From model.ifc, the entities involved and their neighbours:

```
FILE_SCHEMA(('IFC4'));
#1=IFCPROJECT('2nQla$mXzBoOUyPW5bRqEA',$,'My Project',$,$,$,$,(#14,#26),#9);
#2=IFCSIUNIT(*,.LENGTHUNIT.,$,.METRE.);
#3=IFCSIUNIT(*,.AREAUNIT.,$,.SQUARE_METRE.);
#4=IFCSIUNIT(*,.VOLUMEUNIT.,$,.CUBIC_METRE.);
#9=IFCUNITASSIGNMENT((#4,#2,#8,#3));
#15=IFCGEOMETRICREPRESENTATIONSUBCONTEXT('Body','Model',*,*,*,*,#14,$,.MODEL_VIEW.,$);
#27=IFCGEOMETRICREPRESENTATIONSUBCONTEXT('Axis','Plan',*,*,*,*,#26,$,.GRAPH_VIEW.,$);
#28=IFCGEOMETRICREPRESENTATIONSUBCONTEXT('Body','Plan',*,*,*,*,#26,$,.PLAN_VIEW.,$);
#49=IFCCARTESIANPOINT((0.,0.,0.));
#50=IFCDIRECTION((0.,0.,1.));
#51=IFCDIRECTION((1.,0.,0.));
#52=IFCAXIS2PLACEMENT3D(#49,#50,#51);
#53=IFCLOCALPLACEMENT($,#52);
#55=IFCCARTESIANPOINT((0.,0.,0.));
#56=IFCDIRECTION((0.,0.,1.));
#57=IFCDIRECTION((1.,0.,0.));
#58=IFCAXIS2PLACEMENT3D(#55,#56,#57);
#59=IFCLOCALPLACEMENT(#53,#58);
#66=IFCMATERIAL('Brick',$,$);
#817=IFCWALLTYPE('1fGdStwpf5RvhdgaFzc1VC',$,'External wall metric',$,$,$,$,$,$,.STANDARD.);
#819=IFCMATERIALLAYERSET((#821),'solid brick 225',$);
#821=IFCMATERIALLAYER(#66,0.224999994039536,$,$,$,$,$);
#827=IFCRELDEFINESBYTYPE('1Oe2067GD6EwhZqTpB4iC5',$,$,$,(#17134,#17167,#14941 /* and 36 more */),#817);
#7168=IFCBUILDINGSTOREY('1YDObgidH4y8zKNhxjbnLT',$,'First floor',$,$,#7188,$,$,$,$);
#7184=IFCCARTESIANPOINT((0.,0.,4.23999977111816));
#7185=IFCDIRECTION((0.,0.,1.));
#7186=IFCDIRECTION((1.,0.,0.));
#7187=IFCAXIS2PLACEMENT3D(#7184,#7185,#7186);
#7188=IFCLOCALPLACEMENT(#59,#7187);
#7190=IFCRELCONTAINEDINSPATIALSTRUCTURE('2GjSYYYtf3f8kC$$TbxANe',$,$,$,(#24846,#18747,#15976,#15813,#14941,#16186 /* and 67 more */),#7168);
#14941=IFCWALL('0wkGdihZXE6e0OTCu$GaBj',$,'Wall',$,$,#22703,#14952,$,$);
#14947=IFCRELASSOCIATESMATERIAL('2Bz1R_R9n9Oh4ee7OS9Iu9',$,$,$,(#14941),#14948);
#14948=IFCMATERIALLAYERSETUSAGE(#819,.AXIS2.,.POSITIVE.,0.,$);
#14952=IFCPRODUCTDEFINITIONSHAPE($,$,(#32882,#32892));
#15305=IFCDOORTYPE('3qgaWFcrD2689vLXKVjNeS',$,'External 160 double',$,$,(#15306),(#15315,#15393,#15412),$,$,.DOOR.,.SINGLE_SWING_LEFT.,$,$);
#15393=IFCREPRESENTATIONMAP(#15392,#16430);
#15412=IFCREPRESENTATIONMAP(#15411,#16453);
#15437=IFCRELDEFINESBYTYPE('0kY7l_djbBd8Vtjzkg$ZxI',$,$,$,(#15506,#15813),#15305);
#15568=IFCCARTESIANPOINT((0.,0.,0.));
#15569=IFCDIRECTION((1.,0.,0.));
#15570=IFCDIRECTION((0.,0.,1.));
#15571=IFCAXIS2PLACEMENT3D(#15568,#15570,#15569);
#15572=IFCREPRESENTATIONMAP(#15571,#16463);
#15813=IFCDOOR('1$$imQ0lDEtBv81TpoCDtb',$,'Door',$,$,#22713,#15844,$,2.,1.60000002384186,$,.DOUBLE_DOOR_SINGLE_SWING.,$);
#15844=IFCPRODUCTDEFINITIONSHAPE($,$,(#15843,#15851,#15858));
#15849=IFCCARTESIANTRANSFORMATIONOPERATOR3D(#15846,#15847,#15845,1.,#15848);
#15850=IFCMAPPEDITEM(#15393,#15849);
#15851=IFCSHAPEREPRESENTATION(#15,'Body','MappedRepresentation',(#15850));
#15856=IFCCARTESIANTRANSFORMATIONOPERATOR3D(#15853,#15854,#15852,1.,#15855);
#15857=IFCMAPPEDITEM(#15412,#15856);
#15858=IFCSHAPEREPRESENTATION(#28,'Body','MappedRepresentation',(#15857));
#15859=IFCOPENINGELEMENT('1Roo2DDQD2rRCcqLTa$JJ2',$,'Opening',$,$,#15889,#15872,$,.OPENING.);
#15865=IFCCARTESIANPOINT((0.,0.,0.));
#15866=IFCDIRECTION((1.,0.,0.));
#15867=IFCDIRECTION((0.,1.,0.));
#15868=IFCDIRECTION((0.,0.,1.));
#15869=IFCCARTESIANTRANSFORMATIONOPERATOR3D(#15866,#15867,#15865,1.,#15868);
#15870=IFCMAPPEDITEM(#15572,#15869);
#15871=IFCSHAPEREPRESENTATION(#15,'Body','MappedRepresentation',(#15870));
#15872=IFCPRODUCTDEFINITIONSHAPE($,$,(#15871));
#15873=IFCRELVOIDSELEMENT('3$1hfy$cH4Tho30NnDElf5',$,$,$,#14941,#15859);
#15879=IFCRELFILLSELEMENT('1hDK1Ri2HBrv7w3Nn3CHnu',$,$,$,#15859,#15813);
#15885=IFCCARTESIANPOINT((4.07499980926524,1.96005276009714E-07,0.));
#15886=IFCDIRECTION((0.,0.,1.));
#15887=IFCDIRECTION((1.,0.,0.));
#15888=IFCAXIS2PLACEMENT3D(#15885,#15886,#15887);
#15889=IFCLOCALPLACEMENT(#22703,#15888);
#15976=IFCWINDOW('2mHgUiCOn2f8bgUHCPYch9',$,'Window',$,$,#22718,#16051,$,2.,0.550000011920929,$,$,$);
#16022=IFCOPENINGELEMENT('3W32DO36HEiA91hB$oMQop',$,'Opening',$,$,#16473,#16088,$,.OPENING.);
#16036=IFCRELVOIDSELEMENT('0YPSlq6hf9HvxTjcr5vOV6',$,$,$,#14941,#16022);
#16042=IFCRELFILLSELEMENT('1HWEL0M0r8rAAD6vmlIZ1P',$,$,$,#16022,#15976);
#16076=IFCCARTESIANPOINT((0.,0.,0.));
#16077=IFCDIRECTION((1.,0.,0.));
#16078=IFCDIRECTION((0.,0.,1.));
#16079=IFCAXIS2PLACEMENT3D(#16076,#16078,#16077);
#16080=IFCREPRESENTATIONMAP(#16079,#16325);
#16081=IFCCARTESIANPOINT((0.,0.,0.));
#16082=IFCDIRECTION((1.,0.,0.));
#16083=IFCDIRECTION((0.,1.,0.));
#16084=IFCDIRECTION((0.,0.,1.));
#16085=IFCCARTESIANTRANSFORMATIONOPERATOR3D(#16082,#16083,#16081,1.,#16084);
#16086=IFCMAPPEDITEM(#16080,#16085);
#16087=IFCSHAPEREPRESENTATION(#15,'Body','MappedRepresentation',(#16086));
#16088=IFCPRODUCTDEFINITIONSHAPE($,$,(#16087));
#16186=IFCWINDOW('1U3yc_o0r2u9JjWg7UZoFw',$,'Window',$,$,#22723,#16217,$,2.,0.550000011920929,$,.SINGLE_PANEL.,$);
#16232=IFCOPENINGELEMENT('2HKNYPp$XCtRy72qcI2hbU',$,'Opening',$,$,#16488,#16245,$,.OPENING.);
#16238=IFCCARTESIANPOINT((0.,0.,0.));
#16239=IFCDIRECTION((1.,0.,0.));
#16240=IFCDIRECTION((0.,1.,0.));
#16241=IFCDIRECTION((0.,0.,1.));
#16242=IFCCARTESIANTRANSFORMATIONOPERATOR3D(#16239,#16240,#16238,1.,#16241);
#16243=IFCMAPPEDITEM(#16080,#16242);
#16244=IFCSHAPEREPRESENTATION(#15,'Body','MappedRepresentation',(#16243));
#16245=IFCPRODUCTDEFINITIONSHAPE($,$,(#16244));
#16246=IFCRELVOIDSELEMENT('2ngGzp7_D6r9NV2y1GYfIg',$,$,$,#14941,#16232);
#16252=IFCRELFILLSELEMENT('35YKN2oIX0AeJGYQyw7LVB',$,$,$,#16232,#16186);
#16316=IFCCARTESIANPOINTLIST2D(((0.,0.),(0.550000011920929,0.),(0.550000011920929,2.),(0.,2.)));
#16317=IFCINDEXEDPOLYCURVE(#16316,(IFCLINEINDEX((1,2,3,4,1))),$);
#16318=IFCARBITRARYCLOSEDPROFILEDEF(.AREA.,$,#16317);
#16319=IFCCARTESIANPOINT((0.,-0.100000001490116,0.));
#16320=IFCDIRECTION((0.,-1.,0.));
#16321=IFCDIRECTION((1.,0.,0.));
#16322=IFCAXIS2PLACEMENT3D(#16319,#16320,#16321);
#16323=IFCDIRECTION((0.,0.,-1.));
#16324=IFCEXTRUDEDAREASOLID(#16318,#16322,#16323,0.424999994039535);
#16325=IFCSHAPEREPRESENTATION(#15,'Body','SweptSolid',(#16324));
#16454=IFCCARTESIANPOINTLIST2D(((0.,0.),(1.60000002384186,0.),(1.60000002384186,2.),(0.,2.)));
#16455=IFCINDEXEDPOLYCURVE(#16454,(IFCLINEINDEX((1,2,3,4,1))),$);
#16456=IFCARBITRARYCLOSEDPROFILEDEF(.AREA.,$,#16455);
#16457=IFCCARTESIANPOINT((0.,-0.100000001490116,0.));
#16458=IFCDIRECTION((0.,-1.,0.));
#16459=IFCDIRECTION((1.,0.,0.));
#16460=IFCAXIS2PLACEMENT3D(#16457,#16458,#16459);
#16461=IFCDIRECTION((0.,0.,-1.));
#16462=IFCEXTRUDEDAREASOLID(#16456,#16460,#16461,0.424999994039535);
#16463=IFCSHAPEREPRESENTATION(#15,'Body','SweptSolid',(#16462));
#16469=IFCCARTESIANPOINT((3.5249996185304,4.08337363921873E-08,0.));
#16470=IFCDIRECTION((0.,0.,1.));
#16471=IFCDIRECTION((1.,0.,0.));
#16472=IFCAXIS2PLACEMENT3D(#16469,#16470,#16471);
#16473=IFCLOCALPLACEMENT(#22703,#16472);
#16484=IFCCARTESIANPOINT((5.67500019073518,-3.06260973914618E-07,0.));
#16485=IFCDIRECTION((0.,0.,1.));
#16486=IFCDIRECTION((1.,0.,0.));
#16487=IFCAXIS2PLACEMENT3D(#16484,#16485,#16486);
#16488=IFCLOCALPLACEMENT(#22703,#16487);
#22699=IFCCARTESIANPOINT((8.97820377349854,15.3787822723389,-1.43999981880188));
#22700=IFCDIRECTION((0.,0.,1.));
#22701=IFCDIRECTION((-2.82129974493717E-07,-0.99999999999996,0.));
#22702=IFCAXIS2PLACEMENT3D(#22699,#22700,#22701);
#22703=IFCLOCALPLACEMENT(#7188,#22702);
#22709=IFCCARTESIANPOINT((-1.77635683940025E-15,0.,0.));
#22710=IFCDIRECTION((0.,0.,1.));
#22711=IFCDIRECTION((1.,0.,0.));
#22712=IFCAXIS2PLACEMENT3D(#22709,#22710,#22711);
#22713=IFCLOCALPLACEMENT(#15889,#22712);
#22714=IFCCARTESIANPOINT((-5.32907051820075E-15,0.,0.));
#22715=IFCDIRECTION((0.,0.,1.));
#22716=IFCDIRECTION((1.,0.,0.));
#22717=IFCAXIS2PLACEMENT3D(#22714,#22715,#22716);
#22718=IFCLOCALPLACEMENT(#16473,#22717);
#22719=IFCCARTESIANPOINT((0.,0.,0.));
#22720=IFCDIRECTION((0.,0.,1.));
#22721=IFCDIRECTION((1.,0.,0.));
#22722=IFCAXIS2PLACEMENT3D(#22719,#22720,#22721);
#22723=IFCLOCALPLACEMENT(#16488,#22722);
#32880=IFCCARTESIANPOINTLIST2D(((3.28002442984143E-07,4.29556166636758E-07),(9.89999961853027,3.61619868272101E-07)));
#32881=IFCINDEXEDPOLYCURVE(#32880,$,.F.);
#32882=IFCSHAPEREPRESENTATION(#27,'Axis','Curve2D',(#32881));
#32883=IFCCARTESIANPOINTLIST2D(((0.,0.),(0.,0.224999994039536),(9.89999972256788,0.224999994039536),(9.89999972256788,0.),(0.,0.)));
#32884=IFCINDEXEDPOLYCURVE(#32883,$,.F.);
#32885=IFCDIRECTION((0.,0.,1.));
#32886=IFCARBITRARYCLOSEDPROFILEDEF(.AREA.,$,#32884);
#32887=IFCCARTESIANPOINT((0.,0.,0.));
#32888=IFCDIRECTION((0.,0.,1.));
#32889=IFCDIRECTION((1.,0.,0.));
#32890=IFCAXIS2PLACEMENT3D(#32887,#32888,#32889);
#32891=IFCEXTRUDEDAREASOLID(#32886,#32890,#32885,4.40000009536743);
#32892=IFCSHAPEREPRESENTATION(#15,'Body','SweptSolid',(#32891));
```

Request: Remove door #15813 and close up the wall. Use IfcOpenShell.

```python
import ifcopenshell
import ifcopenshell.api.feature
import ifcopenshell.api.root
import ifcopenshell.geom
import ifcopenshell.util.shape

model = ifcopenshell.open("model.ifc")
settings = ifcopenshell.geom.settings()


def volume(element):
    """Net volume in cubic metres, openings subtracted."""
    shape = ifcopenshell.geom.create_shape(settings, element)
    return ifcopenshell.util.shape.get_volume(shape.geometry)


door = model.by_guid("1$$imQ0lDEtBv81TpoCDtb")
opening = door.FillsVoids[0].RelatingOpeningElement
wall = opening.VoidsElements[0].RelatingBuildingElement
before = volume(wall)

ifcopenshell.api.root.remove_product(model, product=door)
ifcopenshell.api.feature.remove_feature(model, feature=opening)

after = volume(wall)

print(f"wall volume {before:.3f} -> {after:.3f} m3")

model.write("model-out.ifc")
```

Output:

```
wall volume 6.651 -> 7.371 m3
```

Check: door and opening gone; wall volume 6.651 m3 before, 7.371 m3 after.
